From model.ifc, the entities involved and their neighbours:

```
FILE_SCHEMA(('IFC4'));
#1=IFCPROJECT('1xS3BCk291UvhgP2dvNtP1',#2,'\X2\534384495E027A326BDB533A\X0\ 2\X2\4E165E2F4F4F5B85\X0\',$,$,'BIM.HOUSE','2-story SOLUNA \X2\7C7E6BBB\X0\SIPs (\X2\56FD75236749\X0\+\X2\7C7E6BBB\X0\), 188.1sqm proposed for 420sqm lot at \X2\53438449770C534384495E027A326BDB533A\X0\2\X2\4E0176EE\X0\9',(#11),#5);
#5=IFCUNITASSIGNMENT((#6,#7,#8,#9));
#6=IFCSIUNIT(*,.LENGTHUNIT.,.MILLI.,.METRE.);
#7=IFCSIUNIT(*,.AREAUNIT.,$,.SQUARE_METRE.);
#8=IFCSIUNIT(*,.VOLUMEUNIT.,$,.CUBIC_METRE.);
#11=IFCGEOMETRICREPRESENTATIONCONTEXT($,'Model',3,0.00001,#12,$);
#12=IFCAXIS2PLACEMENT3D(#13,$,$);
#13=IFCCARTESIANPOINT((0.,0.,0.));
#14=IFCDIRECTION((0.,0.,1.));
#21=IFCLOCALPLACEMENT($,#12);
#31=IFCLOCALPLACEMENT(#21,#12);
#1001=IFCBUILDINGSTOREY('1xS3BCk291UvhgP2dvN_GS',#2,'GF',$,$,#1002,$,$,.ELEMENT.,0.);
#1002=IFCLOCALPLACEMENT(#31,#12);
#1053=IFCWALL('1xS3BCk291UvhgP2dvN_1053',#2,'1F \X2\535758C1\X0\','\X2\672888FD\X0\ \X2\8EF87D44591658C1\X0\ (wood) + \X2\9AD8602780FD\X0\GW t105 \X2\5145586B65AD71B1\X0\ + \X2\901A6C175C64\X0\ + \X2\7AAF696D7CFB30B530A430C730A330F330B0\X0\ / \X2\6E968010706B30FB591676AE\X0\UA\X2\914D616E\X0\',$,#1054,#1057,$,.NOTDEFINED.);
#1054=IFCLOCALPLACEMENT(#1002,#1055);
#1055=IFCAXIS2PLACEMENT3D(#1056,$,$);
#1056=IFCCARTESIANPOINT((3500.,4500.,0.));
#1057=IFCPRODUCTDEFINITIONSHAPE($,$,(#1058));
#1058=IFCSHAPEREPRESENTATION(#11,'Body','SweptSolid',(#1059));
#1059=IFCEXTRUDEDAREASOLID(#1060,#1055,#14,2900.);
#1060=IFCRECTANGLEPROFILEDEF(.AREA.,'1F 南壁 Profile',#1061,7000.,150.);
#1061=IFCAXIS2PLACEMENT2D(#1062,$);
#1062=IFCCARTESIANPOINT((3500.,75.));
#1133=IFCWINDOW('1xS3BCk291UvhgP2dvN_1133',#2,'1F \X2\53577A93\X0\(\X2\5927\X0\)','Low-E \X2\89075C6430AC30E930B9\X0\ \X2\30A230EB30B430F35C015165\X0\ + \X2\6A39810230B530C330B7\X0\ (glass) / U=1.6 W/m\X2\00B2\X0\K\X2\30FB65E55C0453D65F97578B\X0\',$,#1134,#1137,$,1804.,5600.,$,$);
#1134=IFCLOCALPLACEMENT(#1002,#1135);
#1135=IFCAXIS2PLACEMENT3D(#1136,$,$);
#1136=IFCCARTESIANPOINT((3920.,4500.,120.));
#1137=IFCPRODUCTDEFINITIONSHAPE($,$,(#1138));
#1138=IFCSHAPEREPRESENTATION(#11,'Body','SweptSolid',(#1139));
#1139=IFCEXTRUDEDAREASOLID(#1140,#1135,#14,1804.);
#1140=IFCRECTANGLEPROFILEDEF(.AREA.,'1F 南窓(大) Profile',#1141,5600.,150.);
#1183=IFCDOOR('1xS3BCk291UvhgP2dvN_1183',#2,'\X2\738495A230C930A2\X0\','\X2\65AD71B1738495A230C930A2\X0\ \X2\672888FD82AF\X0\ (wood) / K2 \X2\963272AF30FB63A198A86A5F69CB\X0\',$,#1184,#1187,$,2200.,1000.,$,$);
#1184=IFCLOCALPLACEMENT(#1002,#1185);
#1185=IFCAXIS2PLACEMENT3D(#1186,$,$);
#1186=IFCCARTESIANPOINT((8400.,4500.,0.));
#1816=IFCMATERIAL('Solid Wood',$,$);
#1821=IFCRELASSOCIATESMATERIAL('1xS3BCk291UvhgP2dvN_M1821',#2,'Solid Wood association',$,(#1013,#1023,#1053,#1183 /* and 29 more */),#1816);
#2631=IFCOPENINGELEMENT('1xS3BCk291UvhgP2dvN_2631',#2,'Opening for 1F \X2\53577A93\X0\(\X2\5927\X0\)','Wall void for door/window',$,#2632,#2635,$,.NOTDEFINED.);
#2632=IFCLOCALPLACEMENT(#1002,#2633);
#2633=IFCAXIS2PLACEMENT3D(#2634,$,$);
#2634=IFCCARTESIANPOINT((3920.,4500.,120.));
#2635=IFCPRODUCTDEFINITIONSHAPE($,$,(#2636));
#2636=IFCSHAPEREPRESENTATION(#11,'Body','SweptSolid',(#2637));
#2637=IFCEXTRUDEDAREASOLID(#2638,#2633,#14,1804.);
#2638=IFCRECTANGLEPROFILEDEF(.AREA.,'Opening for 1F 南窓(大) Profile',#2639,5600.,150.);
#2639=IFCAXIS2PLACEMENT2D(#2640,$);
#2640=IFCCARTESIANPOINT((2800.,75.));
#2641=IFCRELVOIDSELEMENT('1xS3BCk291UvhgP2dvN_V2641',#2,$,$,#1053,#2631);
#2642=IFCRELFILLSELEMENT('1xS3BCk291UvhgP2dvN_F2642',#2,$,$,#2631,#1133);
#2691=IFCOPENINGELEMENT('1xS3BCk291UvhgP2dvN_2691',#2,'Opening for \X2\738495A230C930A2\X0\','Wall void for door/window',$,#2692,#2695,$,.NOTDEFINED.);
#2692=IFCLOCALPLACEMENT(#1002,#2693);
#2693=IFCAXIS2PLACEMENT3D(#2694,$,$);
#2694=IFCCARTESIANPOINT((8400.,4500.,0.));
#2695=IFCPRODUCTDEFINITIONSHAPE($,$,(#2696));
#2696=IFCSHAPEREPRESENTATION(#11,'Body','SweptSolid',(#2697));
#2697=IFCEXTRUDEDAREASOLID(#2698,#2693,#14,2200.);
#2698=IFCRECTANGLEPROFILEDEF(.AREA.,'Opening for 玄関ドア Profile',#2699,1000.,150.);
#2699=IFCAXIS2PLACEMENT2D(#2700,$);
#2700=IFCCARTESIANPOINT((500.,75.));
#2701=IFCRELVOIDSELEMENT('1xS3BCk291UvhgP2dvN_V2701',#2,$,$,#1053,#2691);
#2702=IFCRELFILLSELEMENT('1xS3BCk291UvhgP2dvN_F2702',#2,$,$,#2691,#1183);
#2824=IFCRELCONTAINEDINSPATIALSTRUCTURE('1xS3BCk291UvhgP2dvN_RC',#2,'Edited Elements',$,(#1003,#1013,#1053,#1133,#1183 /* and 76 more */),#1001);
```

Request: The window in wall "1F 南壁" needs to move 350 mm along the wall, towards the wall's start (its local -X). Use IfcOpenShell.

```python
import ifcopenshell
import ifcopenshell.api.geometry
import ifcopenshell.util.placement
import ifcopenshell.util.unit

model = ifcopenshell.open("model.ifc")
unit_scale = ifcopenshell.util.unit.calculate_unit_scale(model)

window = model.by_guid("1xS3BCk291UvhgP2dvN_1133")
opening = window.FillsVoids[0].RelatingOpeningElement
wall = opening.VoidsElements[0].RelatingBuildingElement

wall_matrix = ifcopenshell.util.placement.get_local_placement(wall.ObjectPlacement)
shift = wall_matrix[:3, 0] * -0.35 / unit_scale
before = ifcopenshell.util.placement.get_local_placement(window.ObjectPlacement)[:3, 3].copy()

# The window is not placed relative to its opening, so move both.
for product in (opening, window):
    matrix = ifcopenshell.util.placement.get_local_placement(product.ObjectPlacement)
    matrix[:3, 3] += shift
    ifcopenshell.api.geometry.edit_object_placement(model, product=product, matrix=matrix, is_si=False)

after = ifcopenshell.util.placement.get_local_placement(window.ObjectPlacement)[:3, 3]
print("window moved by", (after - before).round(3) + 0.0)

model.write("model_rev.ifc")
```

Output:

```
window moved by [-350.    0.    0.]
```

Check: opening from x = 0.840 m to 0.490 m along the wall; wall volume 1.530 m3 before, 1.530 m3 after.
